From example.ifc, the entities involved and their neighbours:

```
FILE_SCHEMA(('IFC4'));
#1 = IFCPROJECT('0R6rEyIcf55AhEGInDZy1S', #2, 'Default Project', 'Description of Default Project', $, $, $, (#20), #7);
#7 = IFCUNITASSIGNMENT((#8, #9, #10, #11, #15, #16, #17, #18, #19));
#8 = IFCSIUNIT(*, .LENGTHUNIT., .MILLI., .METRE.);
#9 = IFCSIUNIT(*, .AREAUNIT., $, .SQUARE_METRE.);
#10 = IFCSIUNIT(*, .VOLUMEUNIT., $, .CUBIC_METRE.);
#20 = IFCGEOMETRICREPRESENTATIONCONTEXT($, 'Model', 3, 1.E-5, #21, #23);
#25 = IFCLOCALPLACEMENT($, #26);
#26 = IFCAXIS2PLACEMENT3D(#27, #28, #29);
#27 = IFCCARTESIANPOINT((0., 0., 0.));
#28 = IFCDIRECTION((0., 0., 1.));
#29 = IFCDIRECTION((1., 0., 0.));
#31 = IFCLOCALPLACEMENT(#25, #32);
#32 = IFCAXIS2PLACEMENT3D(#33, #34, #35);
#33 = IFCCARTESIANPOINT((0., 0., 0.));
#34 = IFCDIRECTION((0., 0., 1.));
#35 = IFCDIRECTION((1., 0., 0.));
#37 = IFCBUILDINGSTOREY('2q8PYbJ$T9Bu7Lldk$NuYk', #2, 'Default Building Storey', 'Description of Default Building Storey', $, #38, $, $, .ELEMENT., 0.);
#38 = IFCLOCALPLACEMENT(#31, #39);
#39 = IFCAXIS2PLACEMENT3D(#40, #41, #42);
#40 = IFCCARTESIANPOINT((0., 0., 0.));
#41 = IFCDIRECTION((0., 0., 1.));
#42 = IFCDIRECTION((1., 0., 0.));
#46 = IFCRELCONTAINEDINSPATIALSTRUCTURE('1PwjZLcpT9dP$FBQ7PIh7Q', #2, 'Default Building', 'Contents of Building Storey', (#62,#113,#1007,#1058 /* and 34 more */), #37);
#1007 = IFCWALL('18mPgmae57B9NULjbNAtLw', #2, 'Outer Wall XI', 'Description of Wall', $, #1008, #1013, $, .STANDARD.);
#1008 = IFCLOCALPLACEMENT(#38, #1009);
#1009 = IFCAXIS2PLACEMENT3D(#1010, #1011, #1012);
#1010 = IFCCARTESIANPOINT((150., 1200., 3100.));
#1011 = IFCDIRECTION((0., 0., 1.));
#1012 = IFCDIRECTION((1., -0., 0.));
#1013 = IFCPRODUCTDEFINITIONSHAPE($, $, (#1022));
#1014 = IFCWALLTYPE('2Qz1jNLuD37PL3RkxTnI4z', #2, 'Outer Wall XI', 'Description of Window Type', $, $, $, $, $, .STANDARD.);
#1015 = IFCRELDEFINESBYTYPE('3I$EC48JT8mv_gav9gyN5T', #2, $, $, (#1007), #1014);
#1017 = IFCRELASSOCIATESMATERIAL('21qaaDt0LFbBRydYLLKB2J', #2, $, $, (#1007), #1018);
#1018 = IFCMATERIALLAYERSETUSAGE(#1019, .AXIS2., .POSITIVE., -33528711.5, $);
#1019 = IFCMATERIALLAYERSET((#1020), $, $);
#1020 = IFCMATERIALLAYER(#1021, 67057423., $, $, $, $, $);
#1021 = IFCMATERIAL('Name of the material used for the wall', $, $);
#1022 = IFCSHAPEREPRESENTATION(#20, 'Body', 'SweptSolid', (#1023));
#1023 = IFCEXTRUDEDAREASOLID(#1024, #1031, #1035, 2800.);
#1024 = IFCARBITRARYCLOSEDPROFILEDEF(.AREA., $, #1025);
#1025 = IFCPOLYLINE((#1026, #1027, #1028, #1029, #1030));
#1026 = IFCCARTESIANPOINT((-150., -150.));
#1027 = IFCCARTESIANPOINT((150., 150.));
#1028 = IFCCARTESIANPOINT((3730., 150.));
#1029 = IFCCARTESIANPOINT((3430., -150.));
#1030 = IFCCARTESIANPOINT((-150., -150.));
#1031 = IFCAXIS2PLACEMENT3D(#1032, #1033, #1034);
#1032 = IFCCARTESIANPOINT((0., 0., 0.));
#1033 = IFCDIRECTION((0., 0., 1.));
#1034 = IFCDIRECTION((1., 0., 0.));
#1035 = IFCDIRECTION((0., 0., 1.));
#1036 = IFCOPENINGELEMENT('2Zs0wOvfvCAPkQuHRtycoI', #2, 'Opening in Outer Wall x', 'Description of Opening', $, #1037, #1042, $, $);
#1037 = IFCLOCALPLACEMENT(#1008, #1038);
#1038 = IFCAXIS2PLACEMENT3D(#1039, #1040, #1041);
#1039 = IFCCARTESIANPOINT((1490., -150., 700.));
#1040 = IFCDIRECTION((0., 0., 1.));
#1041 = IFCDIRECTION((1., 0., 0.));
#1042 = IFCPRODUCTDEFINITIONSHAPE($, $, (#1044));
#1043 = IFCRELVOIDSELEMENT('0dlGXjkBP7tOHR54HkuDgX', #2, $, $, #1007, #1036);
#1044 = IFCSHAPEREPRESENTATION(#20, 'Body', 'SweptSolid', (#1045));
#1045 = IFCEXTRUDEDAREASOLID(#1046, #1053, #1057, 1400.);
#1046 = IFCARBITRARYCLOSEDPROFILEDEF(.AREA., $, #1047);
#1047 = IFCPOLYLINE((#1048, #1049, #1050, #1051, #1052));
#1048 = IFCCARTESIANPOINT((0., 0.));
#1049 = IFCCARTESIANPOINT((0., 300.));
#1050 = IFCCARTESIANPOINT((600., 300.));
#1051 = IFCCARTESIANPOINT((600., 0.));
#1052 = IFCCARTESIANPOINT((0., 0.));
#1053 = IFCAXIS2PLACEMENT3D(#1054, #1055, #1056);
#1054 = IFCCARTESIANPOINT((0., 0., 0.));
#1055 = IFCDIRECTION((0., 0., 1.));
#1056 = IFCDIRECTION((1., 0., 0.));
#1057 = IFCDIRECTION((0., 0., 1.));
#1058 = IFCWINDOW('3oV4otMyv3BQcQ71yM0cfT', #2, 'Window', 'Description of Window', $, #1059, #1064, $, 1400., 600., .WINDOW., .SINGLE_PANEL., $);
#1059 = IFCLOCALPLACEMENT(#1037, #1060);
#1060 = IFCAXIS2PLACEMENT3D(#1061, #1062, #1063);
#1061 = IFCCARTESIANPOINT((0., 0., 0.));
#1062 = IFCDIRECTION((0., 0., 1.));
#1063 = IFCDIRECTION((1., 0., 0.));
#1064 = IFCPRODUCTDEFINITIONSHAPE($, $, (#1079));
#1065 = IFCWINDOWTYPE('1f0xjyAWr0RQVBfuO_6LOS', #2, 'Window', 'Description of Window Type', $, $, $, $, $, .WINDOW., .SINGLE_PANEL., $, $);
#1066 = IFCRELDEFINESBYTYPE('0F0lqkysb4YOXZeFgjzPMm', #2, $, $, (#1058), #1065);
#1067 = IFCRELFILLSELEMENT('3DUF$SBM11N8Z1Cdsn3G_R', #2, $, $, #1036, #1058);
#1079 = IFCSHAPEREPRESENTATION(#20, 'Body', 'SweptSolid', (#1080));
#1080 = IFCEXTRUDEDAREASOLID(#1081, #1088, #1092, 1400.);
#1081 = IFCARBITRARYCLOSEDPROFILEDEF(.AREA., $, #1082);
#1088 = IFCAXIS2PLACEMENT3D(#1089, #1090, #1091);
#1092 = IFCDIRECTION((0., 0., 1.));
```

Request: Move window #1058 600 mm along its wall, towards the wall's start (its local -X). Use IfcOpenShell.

```python
import ifcopenshell
import ifcopenshell.api.geometry
import ifcopenshell.util.placement

model = ifcopenshell.open("example.ifc")

window = model.by_guid("3oV4otMyv3BQcQ71yM0cfT")
opening = window.FillsVoids[0].RelatingOpeningElement
wall = opening.VoidsElements[0].RelatingBuildingElement

wall_matrix = ifcopenshell.util.placement.get_local_placement(wall.ObjectPlacement)
shift = wall_matrix[:3, 0] * -600.0
before = ifcopenshell.util.placement.get_local_placement(window.ObjectPlacement)[:3, 3].copy()

# The window is placed relative to its opening, so it follows when the opening moves.
matrix = ifcopenshell.util.placement.get_local_placement(opening.ObjectPlacement)
matrix[:3, 3] += shift
ifcopenshell.api.geometry.edit_object_placement(
    model, product=opening, matrix=matrix, is_si=False, should_transform_children=True
)

after = ifcopenshell.util.placement.get_local_placement(window.ObjectPlacement)[:3, 3]
print("window moved by", (after - before).round(3) + 0.0)

model.write("example_rev.ifc")
```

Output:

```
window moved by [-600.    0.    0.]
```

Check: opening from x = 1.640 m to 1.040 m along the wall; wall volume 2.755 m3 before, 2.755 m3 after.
